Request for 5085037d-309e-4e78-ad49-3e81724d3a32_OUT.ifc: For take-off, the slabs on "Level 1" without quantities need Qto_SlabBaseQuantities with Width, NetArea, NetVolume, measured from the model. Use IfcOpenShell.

First a look at what the model holds.

```python
import ifcopenshell
import ifcopenshell.util.element
import ifcopenshell.util.unit

model = ifcopenshell.open("5085037d-309e-4e78-ad49-3e81724d3a32_OUT.ifc")
print(model.schema)
for unit_type in ("LENGTHUNIT", "AREAUNIT", "VOLUMEUNIT"):
    print(unit_type, ifcopenshell.util.unit.calculate_unit_scale(model, unit_type))
storey = next(s for s in model.by_type("IfcBuildingStorey") if s.Name == "Level 1")
slabs = [e for e in ifcopenshell.util.element.get_decomposition(storey) if e.is_a("IfcSlab")]
for e in sorted(slabs, key=lambda e: e.id()):
    print(e.id(), e.is_a(), e.Name, list(ifcopenshell.util.element.get_psets(e, qtos_only=True)), sep=" | ")
```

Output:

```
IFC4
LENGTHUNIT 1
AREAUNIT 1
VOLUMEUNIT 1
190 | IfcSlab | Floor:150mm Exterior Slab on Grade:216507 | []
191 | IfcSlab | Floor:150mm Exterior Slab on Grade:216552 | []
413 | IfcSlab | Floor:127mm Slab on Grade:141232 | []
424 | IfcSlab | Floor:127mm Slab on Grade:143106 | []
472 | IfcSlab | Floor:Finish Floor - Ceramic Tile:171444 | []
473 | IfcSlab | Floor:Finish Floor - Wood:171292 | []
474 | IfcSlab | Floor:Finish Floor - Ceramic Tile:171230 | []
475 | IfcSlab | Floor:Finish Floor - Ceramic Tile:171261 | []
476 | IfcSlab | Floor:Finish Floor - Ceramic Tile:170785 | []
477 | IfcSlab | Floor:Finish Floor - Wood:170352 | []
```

```python
import ifcopenshell
import ifcopenshell.api.pset
import ifcopenshell.geom
import ifcopenshell.util.element
import ifcopenshell.util.shape
import ifcopenshell.util.unit

model = ifcopenshell.open("5085037d-309e-4e78-ad49-3e81724d3a32_OUT.ifc")
unit_scale = ifcopenshell.util.unit.calculate_unit_scale(model)
area_scale = ifcopenshell.util.unit.calculate_unit_scale(model, "AREAUNIT")
volume_scale = ifcopenshell.util.unit.calculate_unit_scale(model, "VOLUMEUNIT")
settings = ifcopenshell.geom.settings()

storey = next(s for s in model.by_type("IfcBuildingStorey") if s.Name == "Level 1")
slabs = [e for e in ifcopenshell.util.element.get_decomposition(storey) if e.is_a("IfcSlab")]

for e in sorted(slabs, key=lambda e: e.id()):
    if ifcopenshell.util.element.get_psets(e, qtos_only=True, should_inherit=False):
        continue
    # Geometry comes back in metres, in the element's own axes.
    shape = ifcopenshell.geom.create_shape(settings, e)
    values = {
        "Width": ifcopenshell.util.shape.get_z(shape.geometry) / unit_scale,
        "NetArea": ifcopenshell.util.shape.get_footprint_area(shape.geometry) / area_scale,
        "NetVolume": ifcopenshell.util.shape.get_volume(shape.geometry) / volume_scale,
    }
    qto = ifcopenshell.api.pset.add_qto(model, product=e, name="Qto_SlabBaseQuantities")
    ifcopenshell.api.pset.edit_qto(model, qto=qto, properties=values)
    print(e.id(), {k: round(v, 3) for k, v in values.items()})

model.write("5085037d-309e-4e78-ad49-3e81724d3a32_OUT_edited.ifc")
```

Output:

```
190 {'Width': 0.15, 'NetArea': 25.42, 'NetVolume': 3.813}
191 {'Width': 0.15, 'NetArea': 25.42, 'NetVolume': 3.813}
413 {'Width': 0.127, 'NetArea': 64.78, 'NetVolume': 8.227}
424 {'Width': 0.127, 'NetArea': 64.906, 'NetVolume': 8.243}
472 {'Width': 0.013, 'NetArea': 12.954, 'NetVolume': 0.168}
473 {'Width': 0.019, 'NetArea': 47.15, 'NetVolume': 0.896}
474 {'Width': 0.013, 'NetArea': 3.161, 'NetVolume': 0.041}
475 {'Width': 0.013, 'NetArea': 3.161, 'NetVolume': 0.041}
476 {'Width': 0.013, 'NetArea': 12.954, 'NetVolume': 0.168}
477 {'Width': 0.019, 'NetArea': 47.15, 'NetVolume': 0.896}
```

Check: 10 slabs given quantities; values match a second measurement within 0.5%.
